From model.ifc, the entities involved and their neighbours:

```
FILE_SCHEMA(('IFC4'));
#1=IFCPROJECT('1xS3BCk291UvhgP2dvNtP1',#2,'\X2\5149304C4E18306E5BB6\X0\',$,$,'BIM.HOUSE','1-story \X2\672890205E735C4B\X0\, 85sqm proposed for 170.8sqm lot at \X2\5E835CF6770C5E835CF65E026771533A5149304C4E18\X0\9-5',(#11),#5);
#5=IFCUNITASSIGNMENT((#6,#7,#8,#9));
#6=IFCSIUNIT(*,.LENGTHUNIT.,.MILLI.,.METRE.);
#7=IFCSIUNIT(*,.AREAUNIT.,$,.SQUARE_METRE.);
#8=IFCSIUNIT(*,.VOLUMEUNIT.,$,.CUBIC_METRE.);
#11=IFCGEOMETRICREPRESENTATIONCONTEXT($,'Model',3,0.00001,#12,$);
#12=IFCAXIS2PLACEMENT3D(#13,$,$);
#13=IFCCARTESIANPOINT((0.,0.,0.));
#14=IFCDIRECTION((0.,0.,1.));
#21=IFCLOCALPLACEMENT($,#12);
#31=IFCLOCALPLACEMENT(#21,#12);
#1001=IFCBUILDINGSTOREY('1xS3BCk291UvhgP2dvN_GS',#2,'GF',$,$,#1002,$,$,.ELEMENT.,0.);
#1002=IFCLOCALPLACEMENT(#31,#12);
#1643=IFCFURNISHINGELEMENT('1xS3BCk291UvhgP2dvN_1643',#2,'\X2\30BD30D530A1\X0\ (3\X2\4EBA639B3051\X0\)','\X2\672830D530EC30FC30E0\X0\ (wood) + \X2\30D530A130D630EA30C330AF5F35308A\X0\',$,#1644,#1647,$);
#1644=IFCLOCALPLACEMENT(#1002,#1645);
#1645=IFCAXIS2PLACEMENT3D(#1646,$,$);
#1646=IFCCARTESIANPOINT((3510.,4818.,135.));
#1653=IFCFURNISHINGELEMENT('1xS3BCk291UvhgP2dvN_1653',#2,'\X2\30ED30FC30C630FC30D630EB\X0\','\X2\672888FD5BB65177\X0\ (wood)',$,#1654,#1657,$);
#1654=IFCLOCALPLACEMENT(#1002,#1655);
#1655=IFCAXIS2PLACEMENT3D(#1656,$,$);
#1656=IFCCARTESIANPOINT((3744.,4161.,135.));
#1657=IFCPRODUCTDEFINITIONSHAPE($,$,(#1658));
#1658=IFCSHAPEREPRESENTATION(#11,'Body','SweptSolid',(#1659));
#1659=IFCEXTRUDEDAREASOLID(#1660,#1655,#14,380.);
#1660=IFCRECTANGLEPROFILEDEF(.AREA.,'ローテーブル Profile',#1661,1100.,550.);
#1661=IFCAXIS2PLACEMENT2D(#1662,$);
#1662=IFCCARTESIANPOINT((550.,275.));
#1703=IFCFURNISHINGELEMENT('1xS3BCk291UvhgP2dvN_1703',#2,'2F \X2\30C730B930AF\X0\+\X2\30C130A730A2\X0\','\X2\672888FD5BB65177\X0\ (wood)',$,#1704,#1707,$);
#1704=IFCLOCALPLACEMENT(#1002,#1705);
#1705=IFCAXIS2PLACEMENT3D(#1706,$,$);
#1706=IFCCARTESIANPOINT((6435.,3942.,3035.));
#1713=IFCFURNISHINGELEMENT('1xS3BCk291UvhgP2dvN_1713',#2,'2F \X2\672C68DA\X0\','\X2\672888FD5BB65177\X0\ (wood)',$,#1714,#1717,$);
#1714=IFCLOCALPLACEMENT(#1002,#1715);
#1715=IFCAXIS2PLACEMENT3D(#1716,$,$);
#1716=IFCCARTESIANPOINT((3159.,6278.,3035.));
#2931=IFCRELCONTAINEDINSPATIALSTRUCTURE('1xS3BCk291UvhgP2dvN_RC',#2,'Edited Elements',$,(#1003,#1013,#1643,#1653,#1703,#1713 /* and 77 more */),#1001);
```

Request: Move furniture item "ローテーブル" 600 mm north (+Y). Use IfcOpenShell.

```python
import ifcopenshell
import ifcopenshell.api.geometry
import ifcopenshell.util.placement
import ifcopenshell.util.unit

model = ifcopenshell.open("model.ifc")
unit_scale = ifcopenshell.util.unit.calculate_unit_scale(model)

item = model.by_guid("1xS3BCk291UvhgP2dvN_1653")
matrix = ifcopenshell.util.placement.get_local_placement(item.ObjectPlacement)
matrix[1, 3] += 0.6 / unit_scale
ifcopenshell.api.geometry.edit_object_placement(model, product=item, matrix=matrix, is_si=False)

print(ifcopenshell.util.placement.get_local_placement(item.ObjectPlacement).round(3) + 0.0)

model.write("model_rev.ifc")
```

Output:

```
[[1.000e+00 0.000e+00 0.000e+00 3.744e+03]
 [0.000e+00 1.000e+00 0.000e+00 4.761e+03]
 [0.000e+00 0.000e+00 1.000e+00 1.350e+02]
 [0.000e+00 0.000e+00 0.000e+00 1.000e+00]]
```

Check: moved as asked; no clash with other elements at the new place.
